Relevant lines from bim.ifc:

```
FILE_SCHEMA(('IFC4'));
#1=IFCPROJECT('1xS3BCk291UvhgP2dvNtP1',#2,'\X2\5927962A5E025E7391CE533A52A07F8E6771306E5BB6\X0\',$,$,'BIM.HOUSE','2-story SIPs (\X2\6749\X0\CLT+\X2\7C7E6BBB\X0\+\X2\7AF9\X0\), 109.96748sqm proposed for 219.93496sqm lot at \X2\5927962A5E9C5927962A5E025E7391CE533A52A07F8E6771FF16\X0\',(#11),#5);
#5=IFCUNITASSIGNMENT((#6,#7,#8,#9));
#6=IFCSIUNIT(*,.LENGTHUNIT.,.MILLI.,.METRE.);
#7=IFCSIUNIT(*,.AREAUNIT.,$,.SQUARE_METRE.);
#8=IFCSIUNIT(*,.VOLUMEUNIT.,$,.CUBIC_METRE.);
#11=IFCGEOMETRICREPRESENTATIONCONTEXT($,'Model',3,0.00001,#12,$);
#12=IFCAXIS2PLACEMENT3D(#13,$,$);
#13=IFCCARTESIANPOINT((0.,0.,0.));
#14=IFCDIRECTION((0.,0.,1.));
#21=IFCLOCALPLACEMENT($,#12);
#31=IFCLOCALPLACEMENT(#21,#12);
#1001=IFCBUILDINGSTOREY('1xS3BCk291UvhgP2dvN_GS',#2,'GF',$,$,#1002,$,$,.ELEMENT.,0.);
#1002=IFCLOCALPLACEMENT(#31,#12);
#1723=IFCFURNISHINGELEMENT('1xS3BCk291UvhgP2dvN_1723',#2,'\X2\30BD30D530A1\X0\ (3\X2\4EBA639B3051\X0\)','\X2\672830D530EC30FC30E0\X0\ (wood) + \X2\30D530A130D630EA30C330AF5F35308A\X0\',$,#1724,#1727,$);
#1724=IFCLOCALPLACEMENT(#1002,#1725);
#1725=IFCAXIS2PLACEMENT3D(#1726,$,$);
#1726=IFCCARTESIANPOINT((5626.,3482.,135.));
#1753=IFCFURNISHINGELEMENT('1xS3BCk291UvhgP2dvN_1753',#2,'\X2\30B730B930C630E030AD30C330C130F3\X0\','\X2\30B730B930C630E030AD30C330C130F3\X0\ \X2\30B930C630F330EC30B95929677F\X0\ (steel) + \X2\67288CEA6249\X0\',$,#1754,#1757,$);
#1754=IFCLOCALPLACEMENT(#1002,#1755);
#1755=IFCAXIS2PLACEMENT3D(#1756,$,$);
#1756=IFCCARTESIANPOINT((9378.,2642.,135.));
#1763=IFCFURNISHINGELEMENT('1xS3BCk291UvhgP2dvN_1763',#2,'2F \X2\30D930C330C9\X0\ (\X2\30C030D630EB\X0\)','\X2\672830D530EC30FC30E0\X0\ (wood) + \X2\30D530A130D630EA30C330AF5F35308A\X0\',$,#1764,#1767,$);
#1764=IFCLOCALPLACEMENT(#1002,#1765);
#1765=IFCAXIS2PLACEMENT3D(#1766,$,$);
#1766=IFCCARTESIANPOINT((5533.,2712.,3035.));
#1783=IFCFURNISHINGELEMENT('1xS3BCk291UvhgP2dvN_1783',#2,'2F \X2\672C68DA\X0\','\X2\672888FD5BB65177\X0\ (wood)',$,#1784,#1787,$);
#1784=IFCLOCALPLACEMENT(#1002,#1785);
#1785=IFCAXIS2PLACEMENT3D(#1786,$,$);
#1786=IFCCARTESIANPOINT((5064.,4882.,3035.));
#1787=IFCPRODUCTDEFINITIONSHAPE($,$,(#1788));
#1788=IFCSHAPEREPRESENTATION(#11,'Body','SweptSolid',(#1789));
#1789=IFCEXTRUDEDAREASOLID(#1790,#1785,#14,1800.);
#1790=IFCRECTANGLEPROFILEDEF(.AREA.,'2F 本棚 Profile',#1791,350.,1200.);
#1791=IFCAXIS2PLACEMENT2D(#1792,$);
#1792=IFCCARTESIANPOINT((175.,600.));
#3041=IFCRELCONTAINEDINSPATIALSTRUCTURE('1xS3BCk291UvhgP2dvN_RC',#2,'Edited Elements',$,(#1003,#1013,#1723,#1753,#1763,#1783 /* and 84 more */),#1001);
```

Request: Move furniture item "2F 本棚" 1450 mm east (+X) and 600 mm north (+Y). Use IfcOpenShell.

```python
import ifcopenshell
import ifcopenshell.api.geometry
import ifcopenshell.util.placement
import ifcopenshell.util.unit

model = ifcopenshell.open("bim.ifc")
unit_scale = ifcopenshell.util.unit.calculate_unit_scale(model)

item = model.by_guid("1xS3BCk291UvhgP2dvN_1783")
matrix = ifcopenshell.util.placement.get_local_placement(item.ObjectPlacement)
matrix[0, 3] += 1.45 / unit_scale
matrix[1, 3] += 0.6 / unit_scale
ifcopenshell.api.geometry.edit_object_placement(model, product=item, matrix=matrix, is_si=False)

print(ifcopenshell.util.placement.get_local_placement(item.ObjectPlacement).round(3) + 0.0)

model.write("bim-out.ifc")
```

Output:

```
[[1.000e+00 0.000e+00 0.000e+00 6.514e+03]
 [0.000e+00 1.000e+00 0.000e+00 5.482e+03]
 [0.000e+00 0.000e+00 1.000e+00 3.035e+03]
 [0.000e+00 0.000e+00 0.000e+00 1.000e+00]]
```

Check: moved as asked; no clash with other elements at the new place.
